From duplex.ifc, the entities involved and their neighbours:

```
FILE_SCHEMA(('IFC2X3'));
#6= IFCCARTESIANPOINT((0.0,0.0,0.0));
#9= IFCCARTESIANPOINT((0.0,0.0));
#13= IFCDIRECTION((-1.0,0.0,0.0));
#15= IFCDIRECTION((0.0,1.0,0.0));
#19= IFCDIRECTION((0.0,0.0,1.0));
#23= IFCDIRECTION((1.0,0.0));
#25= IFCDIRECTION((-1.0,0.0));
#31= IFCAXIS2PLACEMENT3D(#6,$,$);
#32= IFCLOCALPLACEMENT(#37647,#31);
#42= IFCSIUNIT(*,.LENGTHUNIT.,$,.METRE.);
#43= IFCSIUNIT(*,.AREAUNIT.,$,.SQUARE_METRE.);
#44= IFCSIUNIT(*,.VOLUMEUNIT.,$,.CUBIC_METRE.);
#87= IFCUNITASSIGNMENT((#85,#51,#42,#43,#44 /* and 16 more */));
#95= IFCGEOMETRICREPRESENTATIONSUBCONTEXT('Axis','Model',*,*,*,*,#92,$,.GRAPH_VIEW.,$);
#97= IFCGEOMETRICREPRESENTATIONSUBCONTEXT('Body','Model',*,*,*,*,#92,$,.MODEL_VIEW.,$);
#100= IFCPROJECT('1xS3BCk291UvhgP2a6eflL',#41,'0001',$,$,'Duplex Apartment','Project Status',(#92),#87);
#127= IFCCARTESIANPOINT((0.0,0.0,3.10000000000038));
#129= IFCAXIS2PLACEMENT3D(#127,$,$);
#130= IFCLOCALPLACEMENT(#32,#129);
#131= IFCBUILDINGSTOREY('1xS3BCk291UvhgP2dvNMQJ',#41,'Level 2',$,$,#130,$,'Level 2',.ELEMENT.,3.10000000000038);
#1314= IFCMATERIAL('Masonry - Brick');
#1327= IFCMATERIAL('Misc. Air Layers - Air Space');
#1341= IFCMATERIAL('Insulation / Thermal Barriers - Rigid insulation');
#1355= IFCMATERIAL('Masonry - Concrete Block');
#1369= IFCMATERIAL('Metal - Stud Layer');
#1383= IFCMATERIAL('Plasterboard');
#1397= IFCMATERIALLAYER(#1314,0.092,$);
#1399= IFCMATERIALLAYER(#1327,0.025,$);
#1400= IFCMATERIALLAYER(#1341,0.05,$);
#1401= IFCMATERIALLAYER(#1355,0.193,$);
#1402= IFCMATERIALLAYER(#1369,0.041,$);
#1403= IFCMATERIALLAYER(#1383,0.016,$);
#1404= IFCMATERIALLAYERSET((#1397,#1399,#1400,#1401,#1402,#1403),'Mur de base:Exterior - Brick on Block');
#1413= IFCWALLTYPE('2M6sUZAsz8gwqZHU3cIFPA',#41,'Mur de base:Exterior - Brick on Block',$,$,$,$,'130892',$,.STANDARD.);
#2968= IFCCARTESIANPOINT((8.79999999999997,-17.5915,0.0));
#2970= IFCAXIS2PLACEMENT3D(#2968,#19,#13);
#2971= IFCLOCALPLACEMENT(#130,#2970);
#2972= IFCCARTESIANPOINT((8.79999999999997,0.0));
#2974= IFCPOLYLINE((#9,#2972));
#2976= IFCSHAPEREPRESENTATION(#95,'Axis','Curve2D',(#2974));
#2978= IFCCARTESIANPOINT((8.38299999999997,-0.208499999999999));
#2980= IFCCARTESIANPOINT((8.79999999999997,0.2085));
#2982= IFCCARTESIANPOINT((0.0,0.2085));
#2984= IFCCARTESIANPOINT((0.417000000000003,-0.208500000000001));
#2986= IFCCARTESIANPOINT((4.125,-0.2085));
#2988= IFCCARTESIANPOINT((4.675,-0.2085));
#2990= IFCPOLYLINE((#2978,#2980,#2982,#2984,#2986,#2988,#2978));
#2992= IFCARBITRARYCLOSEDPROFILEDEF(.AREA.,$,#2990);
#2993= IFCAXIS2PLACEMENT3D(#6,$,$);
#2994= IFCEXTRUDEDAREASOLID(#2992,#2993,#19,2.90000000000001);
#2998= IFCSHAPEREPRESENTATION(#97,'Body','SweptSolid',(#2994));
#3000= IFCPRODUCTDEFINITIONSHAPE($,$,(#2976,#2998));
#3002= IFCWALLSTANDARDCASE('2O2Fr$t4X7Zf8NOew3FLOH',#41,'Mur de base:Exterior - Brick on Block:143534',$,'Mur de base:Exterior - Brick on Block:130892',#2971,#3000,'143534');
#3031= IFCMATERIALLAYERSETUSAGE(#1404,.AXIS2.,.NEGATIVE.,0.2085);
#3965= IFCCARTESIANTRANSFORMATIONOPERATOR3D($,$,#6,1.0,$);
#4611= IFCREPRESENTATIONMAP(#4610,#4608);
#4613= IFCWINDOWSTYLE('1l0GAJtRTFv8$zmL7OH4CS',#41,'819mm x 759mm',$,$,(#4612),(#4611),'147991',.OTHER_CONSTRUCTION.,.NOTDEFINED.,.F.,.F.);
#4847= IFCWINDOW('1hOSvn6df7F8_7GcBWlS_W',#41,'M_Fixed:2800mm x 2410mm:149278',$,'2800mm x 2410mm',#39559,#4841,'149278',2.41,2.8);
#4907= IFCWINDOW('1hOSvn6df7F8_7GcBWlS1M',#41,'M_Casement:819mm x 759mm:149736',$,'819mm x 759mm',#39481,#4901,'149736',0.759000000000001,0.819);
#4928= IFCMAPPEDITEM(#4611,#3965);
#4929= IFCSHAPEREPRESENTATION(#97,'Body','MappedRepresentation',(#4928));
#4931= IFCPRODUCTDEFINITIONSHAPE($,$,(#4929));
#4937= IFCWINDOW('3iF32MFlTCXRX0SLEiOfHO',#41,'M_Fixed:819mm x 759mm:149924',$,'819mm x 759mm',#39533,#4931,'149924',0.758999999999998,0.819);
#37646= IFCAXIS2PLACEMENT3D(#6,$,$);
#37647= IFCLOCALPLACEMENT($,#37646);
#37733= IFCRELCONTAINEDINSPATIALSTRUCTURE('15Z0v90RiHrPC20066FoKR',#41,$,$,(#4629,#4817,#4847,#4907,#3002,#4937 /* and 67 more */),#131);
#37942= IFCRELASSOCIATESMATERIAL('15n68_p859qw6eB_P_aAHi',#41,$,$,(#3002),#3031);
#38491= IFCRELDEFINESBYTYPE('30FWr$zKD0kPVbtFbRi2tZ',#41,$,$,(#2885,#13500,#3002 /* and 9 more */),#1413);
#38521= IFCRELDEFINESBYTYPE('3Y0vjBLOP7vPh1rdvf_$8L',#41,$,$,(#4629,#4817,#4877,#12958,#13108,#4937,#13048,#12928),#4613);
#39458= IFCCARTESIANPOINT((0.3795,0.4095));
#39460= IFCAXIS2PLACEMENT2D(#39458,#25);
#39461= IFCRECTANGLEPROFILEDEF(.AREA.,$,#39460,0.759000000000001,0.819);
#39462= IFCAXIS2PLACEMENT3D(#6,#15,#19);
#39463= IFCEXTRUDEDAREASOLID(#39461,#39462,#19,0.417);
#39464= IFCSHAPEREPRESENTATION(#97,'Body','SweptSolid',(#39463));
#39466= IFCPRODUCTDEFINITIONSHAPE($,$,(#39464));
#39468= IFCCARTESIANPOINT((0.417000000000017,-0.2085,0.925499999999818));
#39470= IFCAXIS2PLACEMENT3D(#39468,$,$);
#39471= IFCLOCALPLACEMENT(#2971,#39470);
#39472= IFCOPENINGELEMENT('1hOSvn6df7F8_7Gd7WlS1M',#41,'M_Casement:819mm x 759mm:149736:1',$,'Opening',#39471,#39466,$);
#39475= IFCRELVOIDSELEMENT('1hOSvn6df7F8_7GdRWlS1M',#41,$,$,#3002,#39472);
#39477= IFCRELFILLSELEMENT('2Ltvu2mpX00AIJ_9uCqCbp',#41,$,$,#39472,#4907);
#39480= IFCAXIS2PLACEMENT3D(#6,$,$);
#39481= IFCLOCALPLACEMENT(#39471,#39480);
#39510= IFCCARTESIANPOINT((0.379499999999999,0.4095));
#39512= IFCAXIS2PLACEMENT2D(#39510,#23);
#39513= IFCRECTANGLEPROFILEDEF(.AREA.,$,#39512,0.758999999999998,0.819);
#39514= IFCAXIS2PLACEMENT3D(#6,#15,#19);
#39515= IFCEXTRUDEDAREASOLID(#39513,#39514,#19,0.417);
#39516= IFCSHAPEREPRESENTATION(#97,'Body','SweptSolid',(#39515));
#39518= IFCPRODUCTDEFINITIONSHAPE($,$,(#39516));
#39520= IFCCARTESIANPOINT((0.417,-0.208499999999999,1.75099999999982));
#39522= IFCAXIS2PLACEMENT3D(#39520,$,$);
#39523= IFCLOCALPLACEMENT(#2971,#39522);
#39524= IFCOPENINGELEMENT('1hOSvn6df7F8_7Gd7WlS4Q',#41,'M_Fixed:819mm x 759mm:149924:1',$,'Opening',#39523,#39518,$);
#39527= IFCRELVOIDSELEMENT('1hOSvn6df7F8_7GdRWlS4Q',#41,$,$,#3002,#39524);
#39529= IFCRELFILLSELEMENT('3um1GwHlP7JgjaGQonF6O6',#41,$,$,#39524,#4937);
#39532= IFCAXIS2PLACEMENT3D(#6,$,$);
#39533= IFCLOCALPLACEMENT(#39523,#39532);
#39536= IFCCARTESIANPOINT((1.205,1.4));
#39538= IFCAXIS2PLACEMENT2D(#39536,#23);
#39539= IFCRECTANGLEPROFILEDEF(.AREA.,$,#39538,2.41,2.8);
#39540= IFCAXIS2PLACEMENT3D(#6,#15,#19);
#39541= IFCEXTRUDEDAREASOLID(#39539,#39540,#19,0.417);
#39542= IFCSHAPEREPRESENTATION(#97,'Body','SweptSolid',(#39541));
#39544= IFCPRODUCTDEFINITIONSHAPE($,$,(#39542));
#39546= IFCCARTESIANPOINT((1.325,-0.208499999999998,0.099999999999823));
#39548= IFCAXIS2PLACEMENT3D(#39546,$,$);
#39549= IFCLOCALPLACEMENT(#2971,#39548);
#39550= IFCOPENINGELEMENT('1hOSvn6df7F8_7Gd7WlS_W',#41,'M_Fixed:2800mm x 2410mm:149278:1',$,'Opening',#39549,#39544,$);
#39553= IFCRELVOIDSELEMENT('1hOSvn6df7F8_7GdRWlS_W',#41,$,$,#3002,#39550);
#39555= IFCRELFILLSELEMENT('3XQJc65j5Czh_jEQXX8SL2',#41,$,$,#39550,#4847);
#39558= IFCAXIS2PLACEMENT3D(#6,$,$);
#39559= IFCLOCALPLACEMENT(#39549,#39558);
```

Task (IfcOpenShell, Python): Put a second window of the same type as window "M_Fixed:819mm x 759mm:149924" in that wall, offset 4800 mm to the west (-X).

```python
import ifcopenshell
import ifcopenshell.api.feature
import ifcopenshell.api.geometry
import ifcopenshell.api.root
import ifcopenshell.geom
import ifcopenshell.util.element
import ifcopenshell.util.placement
import ifcopenshell.util.shape

model = ifcopenshell.open("duplex.ifc")
settings = ifcopenshell.geom.settings()


def volume(element):
    """Net volume in cubic metres, openings subtracted."""
    shape = ifcopenshell.geom.create_shape(settings, element)
    return ifcopenshell.util.shape.get_volume(shape.geometry)


def reuse_history(source, copy):
    """copy_class also copies each property set's owner history, people and application; keep the originals."""
    for rel in copy.IsDefinedBy:
        if rel.is_a("IfcRelDefinesByProperties") and (history := rel.RelatingPropertyDefinition.OwnerHistory):
            rel.RelatingPropertyDefinition.OwnerHistory = source.OwnerHistory
            ifcopenshell.util.element.remove_deep2(model, history)


window = model.by_guid("3iF32MFlTCXRX0SLEiOfHO")
opening = window.FillsVoids[0].RelatingOpeningElement
wall = opening.VoidsElements[0].RelatingBuildingElement
before = volume(wall)
shift = ifcopenshell.util.placement.get_local_placement(wall.ObjectPlacement)[:3, 0] * 4.8

# copy_class copies the void relationship, type, container and properties, but no geometry.
new_opening = ifcopenshell.api.root.copy_class(model, product=opening)
new_opening.Representation = ifcopenshell.util.element.copy_deep(
    model, opening.Representation, exclude=["IfcGeometricRepresentationContext", "IfcRepresentationMap"]
)
new_opening.Name = "M_Fixed:819mm x 759mm"
new_window = ifcopenshell.api.root.copy_class(model, product=window)
new_window.Representation = ifcopenshell.util.element.copy_deep(
    model, window.Representation, exclude=["IfcGeometricRepresentationContext", "IfcRepresentationMap"]
)
new_window.Name = "M_Fixed:819mm x 759mm"
new_window.Tag = None
reuse_history(window, new_window)
fills = ifcopenshell.api.feature.add_filling(model, opening=new_opening, element=new_window)
fills.OwnerHistory = new_window.OwnerHistory  # required in IFC2X3

for old, new in ((opening, new_opening), (window, new_window)):
    matrix = ifcopenshell.util.placement.get_local_placement(old.ObjectPlacement)
    matrix[:3, 3] += shift
    ifcopenshell.api.geometry.edit_object_placement(model, product=new, matrix=matrix, is_si=False)

after = volume(wall)

print(f"wall volume {before:.3f} -> {after:.3f} m3")

model.write("duplex-out.ifc")
```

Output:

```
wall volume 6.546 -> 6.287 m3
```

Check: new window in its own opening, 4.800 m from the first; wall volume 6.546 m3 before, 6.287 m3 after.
